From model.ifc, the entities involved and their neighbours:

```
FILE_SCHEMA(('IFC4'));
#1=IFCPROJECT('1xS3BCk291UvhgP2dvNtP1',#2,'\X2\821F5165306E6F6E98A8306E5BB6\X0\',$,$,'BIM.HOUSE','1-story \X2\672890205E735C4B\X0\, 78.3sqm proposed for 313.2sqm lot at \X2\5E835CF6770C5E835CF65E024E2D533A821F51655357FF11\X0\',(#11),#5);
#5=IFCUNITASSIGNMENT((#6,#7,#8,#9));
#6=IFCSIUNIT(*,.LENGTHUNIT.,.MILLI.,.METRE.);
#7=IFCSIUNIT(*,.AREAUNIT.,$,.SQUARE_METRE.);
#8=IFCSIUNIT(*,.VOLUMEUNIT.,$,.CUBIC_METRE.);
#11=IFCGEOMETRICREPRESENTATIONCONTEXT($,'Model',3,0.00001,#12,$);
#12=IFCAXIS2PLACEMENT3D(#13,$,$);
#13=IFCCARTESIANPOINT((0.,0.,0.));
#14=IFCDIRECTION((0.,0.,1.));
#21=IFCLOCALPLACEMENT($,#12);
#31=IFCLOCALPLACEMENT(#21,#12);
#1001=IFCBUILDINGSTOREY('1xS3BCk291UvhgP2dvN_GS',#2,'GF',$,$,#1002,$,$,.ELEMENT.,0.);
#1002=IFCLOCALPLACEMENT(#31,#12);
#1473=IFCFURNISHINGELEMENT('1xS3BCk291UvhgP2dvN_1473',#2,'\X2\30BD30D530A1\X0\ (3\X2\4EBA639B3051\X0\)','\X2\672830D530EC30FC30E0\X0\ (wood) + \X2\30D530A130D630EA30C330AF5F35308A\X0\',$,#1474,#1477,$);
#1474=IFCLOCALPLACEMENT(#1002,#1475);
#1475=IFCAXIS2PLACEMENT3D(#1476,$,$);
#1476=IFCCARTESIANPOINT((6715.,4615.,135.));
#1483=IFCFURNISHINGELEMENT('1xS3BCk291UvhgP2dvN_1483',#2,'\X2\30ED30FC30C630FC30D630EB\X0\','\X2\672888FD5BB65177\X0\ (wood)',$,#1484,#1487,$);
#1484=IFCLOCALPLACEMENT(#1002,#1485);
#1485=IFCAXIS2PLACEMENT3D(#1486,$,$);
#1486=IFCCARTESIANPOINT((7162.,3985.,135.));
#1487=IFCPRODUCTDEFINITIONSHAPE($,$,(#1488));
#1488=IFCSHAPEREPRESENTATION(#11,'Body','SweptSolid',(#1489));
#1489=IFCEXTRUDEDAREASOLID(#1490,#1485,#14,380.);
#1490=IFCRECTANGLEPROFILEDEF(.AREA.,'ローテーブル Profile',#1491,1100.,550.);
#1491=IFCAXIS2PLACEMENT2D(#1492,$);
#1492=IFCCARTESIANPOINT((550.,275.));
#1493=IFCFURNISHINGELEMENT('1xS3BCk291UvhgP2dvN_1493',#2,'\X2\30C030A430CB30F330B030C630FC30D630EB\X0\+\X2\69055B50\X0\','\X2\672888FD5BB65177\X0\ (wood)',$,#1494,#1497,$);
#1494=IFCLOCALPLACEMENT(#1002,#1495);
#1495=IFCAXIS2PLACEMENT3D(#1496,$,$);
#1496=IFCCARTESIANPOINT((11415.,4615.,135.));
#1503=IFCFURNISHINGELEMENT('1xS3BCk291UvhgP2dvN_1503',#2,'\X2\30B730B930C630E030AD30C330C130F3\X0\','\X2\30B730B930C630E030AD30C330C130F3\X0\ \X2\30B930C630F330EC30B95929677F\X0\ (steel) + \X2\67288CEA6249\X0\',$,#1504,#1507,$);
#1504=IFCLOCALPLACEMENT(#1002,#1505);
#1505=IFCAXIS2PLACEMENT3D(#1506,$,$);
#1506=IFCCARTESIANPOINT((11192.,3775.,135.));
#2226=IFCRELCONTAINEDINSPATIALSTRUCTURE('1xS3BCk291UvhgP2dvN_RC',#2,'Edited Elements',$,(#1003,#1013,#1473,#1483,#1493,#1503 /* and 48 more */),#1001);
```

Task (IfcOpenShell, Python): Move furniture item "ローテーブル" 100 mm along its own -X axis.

```python
import ifcopenshell
import ifcopenshell.api.geometry
import ifcopenshell.util.placement

model = ifcopenshell.open("model.ifc")

item = model.by_guid("1xS3BCk291UvhgP2dvN_1483")
matrix = ifcopenshell.util.placement.get_local_placement(item.ObjectPlacement)
matrix[:3, 3] -= matrix[:3, 0] * 100.0
ifcopenshell.api.geometry.edit_object_placement(model, product=item, matrix=matrix, is_si=False)

print(ifcopenshell.util.placement.get_local_placement(item.ObjectPlacement).round(3) + 0.0)

model.write("model-out.ifc")
```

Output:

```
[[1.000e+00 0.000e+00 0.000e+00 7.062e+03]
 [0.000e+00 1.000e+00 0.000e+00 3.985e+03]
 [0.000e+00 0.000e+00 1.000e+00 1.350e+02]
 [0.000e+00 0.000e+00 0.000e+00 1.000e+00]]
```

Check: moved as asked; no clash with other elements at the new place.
